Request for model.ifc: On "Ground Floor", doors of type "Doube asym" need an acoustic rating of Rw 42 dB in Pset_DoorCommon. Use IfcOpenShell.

First a look at what the model holds.

```python
import ifcopenshell
import ifcopenshell.util.element

model = ifcopenshell.open("model.ifc")
print(model.schema)
storey = next(s for s in model.by_type("IfcBuildingStorey") if s.Name == "Ground Floor")
doors = [e for e in ifcopenshell.util.element.get_decomposition(storey) if e.is_a("IfcDoor")]
seen = {}
for e in doors:
    element_type = ifcopenshell.util.element.get_type(e)
    key = (element_type.Name if element_type != e and element_type else None, ifcopenshell.util.element.get_pset(e, "Pset_DoorCommon", "AcousticRating"))
    seen[key] = seen.get(key, 0) + 1
for (name, value), count in sorted(seen.items(), key=str):
    print(count, "x", name, "|", value)
```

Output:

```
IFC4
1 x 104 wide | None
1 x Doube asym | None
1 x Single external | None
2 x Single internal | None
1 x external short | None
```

```python
import ifcopenshell
import ifcopenshell.api.pset
import ifcopenshell.util.element

model = ifcopenshell.open("model.ifc")

storey = next(s for s in model.by_type("IfcBuildingStorey") if s.Name == "Ground Floor")
doors = [e for e in ifcopenshell.util.element.get_decomposition(storey) if e.is_a("IfcDoor")]

count = 0
for e in doors:
    element_type = ifcopenshell.util.element.get_type(e)
    if element_type in (None, e) or element_type.Name != "Doube asym":
        continue
    # add_pset returns the element's existing set when there is one.
    pset = ifcopenshell.api.pset.add_pset(model, product=e, name="Pset_DoorCommon")
    ifcopenshell.api.pset.edit_pset(model, pset=pset, properties={"AcousticRating": "Rw 42 dB"})
    count += 1

print(count, "doors updated")

model.write("model_v2.ifc")
```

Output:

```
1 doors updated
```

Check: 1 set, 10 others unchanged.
